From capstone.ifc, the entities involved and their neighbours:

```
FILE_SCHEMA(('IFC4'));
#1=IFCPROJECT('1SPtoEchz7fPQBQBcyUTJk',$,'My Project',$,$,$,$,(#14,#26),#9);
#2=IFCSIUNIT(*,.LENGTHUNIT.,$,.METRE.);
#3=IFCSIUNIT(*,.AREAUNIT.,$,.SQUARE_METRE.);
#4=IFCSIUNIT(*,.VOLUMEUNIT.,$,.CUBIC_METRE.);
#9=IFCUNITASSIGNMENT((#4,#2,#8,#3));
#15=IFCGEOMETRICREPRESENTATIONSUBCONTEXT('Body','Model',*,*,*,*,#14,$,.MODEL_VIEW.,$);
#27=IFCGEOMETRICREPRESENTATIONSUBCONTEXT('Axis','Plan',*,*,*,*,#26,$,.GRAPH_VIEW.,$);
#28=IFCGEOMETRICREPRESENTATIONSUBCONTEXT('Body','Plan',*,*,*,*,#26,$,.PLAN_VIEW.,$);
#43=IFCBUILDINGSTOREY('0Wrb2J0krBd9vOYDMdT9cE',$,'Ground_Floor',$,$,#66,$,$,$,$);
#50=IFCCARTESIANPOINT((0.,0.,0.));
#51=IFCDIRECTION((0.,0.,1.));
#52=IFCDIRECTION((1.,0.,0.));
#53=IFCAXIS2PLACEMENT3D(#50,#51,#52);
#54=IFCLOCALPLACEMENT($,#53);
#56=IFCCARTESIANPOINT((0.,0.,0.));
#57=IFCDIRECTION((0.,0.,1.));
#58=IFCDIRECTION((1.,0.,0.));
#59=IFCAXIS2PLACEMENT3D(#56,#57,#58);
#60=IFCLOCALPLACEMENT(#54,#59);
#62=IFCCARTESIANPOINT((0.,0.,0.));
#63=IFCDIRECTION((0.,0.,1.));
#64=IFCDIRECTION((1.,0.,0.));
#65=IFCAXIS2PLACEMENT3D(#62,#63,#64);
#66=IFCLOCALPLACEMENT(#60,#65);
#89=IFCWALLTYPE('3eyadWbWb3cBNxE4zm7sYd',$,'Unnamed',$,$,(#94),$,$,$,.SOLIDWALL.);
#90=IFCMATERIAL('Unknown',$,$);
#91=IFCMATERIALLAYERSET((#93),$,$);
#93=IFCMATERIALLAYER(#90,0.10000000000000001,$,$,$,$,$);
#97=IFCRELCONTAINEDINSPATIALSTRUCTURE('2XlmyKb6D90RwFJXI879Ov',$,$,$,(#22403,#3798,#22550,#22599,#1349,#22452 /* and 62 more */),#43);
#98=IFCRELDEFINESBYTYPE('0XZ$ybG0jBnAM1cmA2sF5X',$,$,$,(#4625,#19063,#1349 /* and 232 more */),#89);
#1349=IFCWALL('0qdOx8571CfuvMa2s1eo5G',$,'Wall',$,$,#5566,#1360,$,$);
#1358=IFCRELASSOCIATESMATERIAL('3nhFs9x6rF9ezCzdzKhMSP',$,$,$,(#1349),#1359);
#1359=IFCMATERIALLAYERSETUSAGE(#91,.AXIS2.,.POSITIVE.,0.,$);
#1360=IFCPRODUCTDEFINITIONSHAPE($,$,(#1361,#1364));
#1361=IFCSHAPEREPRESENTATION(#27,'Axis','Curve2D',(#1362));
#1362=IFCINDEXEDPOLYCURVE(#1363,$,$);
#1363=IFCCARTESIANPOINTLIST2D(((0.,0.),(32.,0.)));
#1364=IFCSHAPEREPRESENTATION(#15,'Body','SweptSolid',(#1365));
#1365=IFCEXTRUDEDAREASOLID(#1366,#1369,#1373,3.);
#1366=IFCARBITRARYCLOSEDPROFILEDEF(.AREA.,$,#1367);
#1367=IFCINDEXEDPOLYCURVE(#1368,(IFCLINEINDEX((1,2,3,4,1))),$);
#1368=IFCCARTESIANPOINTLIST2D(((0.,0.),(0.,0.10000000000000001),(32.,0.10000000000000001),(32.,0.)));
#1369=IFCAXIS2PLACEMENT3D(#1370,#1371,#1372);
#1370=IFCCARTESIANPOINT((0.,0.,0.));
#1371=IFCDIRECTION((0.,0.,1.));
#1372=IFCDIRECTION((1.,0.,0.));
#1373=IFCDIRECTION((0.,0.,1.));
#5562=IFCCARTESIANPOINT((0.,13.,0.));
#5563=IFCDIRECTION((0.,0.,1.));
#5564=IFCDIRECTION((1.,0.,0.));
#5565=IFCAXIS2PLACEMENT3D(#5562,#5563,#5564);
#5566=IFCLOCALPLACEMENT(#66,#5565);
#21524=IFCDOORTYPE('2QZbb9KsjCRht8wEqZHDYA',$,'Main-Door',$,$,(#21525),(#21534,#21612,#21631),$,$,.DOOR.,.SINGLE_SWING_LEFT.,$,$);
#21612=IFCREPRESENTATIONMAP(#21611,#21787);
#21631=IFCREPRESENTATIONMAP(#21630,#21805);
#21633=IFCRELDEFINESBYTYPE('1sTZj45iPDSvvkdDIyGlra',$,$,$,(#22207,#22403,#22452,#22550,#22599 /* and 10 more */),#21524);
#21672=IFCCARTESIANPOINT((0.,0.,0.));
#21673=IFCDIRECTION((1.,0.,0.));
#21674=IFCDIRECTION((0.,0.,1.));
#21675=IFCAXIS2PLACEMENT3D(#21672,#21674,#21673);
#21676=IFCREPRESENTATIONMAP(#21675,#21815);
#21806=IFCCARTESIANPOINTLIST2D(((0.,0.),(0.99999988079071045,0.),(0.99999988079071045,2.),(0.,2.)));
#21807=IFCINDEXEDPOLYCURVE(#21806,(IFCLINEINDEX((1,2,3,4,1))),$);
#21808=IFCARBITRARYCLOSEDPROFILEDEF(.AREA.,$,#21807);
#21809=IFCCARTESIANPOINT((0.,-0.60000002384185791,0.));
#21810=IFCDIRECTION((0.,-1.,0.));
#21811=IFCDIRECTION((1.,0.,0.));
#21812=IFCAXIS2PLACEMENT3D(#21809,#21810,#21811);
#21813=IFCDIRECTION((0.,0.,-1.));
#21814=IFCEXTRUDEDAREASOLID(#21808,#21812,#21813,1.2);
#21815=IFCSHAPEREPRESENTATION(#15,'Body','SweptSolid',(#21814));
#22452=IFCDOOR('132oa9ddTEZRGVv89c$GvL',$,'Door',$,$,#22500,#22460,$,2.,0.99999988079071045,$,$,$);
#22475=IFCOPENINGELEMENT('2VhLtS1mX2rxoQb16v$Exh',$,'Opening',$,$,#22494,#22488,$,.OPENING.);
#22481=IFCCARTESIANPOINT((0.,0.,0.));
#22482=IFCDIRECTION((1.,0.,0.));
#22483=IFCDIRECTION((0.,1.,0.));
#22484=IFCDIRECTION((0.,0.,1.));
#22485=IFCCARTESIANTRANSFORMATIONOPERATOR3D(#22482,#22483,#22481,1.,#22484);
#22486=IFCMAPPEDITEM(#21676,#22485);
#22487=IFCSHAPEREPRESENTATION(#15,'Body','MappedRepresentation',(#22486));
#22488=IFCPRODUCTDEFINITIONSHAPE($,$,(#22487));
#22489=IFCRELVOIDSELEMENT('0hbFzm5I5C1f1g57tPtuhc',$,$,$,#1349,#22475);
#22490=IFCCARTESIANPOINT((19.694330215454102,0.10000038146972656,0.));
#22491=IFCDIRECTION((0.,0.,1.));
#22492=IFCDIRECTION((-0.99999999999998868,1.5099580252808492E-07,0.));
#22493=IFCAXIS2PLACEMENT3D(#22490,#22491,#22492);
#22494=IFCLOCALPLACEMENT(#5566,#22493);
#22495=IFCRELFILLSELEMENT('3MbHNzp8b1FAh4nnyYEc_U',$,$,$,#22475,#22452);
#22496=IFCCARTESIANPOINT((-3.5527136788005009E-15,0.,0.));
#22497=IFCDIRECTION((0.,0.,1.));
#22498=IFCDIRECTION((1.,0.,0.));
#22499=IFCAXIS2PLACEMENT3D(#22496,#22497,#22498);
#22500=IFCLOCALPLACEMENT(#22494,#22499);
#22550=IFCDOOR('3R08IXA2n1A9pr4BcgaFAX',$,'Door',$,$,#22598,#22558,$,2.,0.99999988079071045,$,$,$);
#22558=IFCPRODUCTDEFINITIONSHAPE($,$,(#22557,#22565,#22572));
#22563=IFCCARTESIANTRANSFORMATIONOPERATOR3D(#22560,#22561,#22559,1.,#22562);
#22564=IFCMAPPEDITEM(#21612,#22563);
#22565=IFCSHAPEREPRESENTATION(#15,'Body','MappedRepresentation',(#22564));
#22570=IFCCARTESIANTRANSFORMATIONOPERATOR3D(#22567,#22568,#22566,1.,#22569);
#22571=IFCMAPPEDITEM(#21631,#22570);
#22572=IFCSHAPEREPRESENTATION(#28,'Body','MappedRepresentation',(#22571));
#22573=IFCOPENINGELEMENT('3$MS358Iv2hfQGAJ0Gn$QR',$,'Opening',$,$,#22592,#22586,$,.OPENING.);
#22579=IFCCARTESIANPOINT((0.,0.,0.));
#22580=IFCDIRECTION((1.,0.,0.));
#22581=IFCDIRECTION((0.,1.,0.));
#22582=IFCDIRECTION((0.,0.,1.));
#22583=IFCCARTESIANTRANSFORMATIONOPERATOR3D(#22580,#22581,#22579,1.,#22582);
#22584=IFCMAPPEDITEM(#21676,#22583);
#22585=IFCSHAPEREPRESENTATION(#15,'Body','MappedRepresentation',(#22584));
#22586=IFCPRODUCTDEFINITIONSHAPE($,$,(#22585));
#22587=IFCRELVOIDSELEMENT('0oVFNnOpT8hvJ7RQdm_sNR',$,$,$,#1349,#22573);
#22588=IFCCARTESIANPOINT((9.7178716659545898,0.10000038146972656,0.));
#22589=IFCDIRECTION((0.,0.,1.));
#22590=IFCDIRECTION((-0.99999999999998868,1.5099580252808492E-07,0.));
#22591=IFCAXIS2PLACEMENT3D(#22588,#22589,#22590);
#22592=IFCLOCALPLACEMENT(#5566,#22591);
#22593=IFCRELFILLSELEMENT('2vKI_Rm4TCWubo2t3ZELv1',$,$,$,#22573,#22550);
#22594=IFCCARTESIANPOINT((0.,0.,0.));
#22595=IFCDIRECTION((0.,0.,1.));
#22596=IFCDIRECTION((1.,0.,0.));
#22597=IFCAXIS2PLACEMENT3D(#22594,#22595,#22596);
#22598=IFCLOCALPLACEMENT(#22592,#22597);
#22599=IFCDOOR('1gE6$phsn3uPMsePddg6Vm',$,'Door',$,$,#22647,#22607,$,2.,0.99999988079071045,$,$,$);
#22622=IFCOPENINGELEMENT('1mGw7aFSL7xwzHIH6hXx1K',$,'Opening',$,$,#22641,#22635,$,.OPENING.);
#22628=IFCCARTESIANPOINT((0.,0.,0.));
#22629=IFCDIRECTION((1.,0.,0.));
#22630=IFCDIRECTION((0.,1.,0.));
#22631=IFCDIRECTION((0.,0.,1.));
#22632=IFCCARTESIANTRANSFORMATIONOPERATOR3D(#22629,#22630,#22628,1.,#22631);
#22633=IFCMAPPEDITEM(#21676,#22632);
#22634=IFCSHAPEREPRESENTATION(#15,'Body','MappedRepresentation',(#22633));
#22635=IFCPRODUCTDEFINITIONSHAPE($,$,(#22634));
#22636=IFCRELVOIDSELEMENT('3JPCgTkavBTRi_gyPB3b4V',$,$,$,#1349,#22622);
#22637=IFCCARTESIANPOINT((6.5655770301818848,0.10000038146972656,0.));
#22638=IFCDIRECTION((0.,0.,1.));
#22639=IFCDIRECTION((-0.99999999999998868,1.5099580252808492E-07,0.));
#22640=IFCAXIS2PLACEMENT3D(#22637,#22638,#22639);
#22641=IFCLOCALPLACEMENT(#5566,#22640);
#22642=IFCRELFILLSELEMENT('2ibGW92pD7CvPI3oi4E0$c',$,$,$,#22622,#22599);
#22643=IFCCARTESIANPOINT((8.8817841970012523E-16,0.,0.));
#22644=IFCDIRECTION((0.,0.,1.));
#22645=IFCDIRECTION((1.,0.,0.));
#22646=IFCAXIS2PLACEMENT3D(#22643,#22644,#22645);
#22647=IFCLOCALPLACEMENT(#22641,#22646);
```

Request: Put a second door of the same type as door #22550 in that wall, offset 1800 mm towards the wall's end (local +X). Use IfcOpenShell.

```python
import ifcopenshell
import ifcopenshell.api.feature
import ifcopenshell.api.geometry
import ifcopenshell.api.root
import ifcopenshell.geom
import ifcopenshell.util.element
import ifcopenshell.util.placement
import ifcopenshell.util.shape
import ifcopenshell.util.unit

model = ifcopenshell.open("capstone.ifc")
unit_scale = ifcopenshell.util.unit.calculate_unit_scale(model)
settings = ifcopenshell.geom.settings()


def volume(element):
    """Net volume in cubic metres, openings subtracted."""
    shape = ifcopenshell.geom.create_shape(settings, element)
    return ifcopenshell.util.shape.get_volume(shape.geometry)


door = model.by_guid("3R08IXA2n1A9pr4BcgaFAX")
opening = door.FillsVoids[0].RelatingOpeningElement
wall = opening.VoidsElements[0].RelatingBuildingElement
before = volume(wall)
shift = ifcopenshell.util.placement.get_local_placement(wall.ObjectPlacement)[:3, 0] * 1.8 / unit_scale

# copy_class copies the void relationship, type, container and properties, but no geometry.
new_opening = ifcopenshell.api.root.copy_class(model, product=opening)
new_opening.Representation = ifcopenshell.util.element.copy_deep(
    model, opening.Representation, exclude=["IfcGeometricRepresentationContext", "IfcRepresentationMap"]
)
new_door = ifcopenshell.api.root.copy_class(model, product=door)
new_door.Representation = ifcopenshell.util.element.copy_deep(
    model, door.Representation, exclude=["IfcGeometricRepresentationContext", "IfcRepresentationMap"]
)
ifcopenshell.api.feature.add_filling(model, opening=new_opening, element=new_door)

for old, new in ((opening, new_opening), (door, new_door)):
    matrix = ifcopenshell.util.placement.get_local_placement(old.ObjectPlacement)
    matrix[:3, 3] += shift
    ifcopenshell.api.geometry.edit_object_placement(model, product=new, matrix=matrix, is_si=False)

after = volume(wall)

print(f"wall volume {before:.3f} -> {after:.3f} m3")

model.write("capstone_rev.ifc")
```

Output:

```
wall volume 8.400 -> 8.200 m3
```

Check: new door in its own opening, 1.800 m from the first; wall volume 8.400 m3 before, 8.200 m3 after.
